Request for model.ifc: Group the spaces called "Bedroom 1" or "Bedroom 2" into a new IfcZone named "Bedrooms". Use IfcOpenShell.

First a look at what the model holds.

```python
import ifcopenshell

model = ifcopenshell.open("model.ifc")
print(model.schema)
seen = {}
for space in model.by_type("IfcSpace"):
    seen[space.LongName] = seen.get(space.LongName, 0) + 1
for name, count in sorted(seen.items(), key=str):
    print(count, "x", name)
print("zones:", [z.Name for z in model.by_type("IfcZone")][:20])
```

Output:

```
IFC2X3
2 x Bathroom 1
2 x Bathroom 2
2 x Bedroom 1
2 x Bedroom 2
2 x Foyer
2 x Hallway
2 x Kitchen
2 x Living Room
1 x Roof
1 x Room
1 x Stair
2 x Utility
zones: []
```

```python
import ifcopenshell
import ifcopenshell.api.group
import ifcopenshell.api.root

model = ifcopenshell.open("model.ifc")

names = {"Bedroom 1", "Bedroom 2"}
spaces = [s for s in model.by_type("IfcSpace") if s.LongName in names]

zone = ifcopenshell.api.root.create_entity(model, ifc_class="IfcZone", name="Bedrooms")
ifcopenshell.api.group.assign_group(model, products=spaces, group=zone)
print(len(spaces), "spaces in", zone.Name)

model.write("model_v2.ifc")
```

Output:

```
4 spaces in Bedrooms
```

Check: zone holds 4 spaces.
